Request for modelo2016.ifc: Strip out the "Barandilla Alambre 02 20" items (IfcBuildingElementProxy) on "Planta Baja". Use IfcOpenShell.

First a look at what the model holds.

```python
import ifcopenshell
import ifcopenshell.util.element

model = ifcopenshell.open("modelo2016.ifc")
print(model.schema)
storey = next(s for s in model.by_type("IfcBuildingStorey") if s.Name == "Planta Baja")
proxies = [e for e in ifcopenshell.util.element.get_decomposition(storey) if e.is_a("IfcBuildingElementProxy")]
seen = {}
for e in proxies:
    element_type = ifcopenshell.util.element.get_type(e)
    name = element_type.Name if element_type not in (None, e) else None
    seen[name] = seen.get(name, 0) + 1
for name, count in sorted(seen.items(), key=str):
    print(count, "x", name)
```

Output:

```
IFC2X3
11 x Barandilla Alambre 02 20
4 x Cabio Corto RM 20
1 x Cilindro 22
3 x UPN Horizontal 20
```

```python
import ifcopenshell
import ifcopenshell.api.root
import ifcopenshell.util.element

model = ifcopenshell.open("modelo2016.ifc")

storey = next(s for s in model.by_type("IfcBuildingStorey") if s.Name == "Planta Baja")
proxies = [e for e in ifcopenshell.util.element.get_decomposition(storey) if e.is_a("IfcBuildingElementProxy")]
targets = [e for e in proxies if (t := ifcopenshell.util.element.get_type(e)) not in (None, e) and t.Name == "Barandilla Alambre 02 20"]

for e in targets:
    ifcopenshell.api.root.remove_product(model, product=e)
print(len(targets), "removed")

model.write("modelo2016_rev.ifc")
```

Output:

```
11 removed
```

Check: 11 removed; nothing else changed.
